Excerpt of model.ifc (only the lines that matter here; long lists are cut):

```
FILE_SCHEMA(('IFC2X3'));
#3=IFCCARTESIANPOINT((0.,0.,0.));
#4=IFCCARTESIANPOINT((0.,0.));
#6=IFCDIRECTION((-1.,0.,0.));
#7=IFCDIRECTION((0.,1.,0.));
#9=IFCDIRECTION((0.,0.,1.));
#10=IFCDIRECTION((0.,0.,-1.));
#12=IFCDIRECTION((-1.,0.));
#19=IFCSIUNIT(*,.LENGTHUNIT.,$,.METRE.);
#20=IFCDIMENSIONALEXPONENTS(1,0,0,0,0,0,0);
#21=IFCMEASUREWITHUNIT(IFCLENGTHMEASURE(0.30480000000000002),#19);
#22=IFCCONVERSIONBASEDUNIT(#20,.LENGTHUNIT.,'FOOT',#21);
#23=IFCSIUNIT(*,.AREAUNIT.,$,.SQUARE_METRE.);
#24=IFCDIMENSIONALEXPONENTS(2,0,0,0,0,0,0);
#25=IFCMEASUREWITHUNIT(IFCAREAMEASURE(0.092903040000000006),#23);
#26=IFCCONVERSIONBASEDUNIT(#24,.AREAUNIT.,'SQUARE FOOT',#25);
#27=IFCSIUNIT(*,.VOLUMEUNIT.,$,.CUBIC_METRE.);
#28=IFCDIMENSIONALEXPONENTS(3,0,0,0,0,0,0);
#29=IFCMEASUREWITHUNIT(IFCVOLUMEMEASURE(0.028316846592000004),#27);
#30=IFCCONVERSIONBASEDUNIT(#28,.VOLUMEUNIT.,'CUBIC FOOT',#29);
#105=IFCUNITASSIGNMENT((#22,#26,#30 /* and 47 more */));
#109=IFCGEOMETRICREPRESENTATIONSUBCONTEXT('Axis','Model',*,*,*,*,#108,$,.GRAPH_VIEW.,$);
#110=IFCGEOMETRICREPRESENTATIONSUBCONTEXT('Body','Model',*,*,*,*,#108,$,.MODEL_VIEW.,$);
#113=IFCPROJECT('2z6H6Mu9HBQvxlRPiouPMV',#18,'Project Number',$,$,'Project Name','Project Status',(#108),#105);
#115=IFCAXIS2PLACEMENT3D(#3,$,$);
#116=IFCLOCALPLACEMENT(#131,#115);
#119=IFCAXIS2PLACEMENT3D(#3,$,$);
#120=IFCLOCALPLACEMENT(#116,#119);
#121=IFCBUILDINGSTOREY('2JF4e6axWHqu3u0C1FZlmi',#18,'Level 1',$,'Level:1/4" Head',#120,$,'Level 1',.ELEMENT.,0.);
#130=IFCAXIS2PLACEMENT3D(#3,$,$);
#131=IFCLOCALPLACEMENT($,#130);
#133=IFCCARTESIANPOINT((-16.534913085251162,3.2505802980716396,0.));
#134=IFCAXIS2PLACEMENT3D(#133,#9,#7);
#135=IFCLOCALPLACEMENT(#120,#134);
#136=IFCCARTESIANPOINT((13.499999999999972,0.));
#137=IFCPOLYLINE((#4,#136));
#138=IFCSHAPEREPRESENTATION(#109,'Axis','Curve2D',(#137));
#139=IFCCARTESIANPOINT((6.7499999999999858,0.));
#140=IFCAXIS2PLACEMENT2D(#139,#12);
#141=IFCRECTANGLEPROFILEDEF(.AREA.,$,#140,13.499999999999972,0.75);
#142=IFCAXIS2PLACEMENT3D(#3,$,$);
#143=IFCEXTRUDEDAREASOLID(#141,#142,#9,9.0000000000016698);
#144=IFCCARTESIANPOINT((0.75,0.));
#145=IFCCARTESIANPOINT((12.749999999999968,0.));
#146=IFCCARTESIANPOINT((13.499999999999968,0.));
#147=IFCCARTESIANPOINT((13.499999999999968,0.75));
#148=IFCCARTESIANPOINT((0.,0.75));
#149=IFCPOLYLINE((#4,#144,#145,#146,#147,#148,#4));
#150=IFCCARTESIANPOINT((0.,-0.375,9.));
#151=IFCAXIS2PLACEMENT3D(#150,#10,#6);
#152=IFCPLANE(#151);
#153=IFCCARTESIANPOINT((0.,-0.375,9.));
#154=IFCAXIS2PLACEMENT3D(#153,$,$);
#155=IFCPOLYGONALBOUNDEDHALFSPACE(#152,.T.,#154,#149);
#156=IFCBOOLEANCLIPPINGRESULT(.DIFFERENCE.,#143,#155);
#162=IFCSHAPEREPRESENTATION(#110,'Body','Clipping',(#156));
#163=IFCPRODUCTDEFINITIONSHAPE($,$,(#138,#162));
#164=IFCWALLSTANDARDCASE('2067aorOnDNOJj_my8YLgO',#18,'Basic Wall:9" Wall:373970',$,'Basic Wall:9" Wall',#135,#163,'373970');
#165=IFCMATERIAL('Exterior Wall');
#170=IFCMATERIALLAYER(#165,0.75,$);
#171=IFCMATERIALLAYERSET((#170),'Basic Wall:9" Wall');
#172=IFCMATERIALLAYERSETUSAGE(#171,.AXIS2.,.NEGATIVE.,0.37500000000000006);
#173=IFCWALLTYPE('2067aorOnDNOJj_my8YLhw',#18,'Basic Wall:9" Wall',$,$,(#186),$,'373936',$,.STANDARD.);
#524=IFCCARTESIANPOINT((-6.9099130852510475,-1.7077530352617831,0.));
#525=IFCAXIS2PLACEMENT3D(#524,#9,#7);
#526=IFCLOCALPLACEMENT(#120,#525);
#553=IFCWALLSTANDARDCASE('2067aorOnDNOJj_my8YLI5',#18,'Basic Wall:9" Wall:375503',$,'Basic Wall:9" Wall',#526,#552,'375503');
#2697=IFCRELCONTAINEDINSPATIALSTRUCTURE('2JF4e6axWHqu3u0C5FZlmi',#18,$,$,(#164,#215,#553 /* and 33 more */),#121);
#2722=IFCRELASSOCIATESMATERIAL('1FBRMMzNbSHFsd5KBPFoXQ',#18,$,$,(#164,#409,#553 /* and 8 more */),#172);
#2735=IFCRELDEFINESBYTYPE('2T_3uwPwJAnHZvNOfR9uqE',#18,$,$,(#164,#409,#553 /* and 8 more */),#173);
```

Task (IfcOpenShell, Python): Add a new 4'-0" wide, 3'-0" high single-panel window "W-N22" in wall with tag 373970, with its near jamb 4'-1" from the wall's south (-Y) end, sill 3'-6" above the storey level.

```python
import numpy as np
import ifcopenshell
import ifcopenshell.api.feature
import ifcopenshell.api.geometry
import ifcopenshell.api.root
import ifcopenshell.api.spatial
import ifcopenshell.api.type
import ifcopenshell.geom
import ifcopenshell.util.element
import ifcopenshell.util.placement
import ifcopenshell.util.representation
import ifcopenshell.util.shape
import ifcopenshell.util.unit

model = ifcopenshell.open("model.ifc")
unit_scale = ifcopenshell.util.unit.calculate_unit_scale(model)
settings = ifcopenshell.geom.settings()


def volume(element):
    """Net volume in cubic metres, openings subtracted."""
    shape = ifcopenshell.geom.create_shape(settings, element)
    return ifcopenshell.util.shape.get_volume(shape.geometry)


wall = model.by_guid("2067aorOnDNOJj_my8YLgO")
storey = ifcopenshell.util.element.get_container(wall, ifc_class="IfcBuildingStorey")
context = ifcopenshell.util.representation.get_context(model, "Model", "Body", "MODEL_VIEW")
before = volume(wall)

width, height, from_end, sill = 1.2192, 0.9144, 1.2446, 1.0668  # metres

# The wall runs along its own X axis, and the end named is its -X end.
wall_shape = ifcopenshell.geom.create_shape(settings, wall)
x, y, z = ifcopenshell.util.shape.get_vertices(wall_shape.geometry).T
start = x.min() + from_end
face, thickness = float(y.min()), float(y.max() - y.min())
wall_matrix = ifcopenshell.util.placement.get_local_placement(wall.ObjectPlacement)
level = ifcopenshell.util.placement.get_local_placement(storey.ObjectPlacement)[2, 3]


def in_wall(x, y):
    """Placement at x, y metres in the wall's axes, at sill height."""
    matrix = wall_matrix.copy()
    matrix[:, 3] = wall_matrix @ np.array([x / unit_scale, y / unit_scale, 0.0, 1.0])
    matrix[2, 3] = level + sill / unit_scale
    return matrix


# Opening: a box that overshoots both wall faces by 50 mm.
opening = ifcopenshell.api.root.create_entity(model, ifc_class="IfcOpeningElement")
box = ifcopenshell.api.geometry.add_wall_representation(
    model, context=context, length=width, height=height, thickness=thickness + 0.1
)
ifcopenshell.api.geometry.assign_representation(model, product=opening, representation=box)
ifcopenshell.api.geometry.edit_object_placement(model, product=opening, matrix=in_wall(start, face - 0.05), is_si=False)
ifcopenshell.api.feature.add_feature(model, feature=opening, element=wall)

window = ifcopenshell.api.root.create_entity(model, ifc_class="IfcWindow", name="W-N22")
window.OverallWidth, window.OverallHeight = width / unit_scale, height / unit_scale
body = ifcopenshell.api.geometry.add_window_representation(
    model,
    context=context,
    overall_width=window.OverallWidth,
    overall_height=window.OverallHeight,
    partition_type="SINGLE_PANEL",
)
ifcopenshell.api.geometry.assign_representation(model, product=window, representation=body)
ifcopenshell.api.spatial.assign_container(model, products=[window], relating_structure=storey)
fills = ifcopenshell.api.feature.add_filling(model, opening=opening, element=window)
fills.OwnerHistory = window.OwnerHistory  # required in IFC2X3

# IFC2X3 keeps the operation on the window style.
style = ifcopenshell.api.root.create_entity(model, ifc_class="IfcWindowStyle", name="W-N22")
style.OperationType, style.ConstructionType = "SINGLE_PANEL", "NOTDEFINED"
style.ParameterTakesPrecedence = style.Sizeable = False
ifcopenshell.api.type.assign_type(model, related_objects=[window], relating_type=style)

# Centre the window in the wall's thickness.
ifcopenshell.api.geometry.edit_object_placement(model, product=window, matrix=in_wall(start, face), is_si=False)
window_shape = ifcopenshell.geom.create_shape(settings, window)
depth = ifcopenshell.util.shape.get_vertices(window_shape.geometry)[:, 1]
offset = face + thickness / 2 - (depth.min() + depth.max()) / 2
ifcopenshell.api.geometry.edit_object_placement(model, product=window, matrix=in_wall(start, offset), is_si=False)

after = volume(wall)

print(f"wall volume {before:.3f} -> {after:.3f} m3")

model.write("model_updated.ifc")
```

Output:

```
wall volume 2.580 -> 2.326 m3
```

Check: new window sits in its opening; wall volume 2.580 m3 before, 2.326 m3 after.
